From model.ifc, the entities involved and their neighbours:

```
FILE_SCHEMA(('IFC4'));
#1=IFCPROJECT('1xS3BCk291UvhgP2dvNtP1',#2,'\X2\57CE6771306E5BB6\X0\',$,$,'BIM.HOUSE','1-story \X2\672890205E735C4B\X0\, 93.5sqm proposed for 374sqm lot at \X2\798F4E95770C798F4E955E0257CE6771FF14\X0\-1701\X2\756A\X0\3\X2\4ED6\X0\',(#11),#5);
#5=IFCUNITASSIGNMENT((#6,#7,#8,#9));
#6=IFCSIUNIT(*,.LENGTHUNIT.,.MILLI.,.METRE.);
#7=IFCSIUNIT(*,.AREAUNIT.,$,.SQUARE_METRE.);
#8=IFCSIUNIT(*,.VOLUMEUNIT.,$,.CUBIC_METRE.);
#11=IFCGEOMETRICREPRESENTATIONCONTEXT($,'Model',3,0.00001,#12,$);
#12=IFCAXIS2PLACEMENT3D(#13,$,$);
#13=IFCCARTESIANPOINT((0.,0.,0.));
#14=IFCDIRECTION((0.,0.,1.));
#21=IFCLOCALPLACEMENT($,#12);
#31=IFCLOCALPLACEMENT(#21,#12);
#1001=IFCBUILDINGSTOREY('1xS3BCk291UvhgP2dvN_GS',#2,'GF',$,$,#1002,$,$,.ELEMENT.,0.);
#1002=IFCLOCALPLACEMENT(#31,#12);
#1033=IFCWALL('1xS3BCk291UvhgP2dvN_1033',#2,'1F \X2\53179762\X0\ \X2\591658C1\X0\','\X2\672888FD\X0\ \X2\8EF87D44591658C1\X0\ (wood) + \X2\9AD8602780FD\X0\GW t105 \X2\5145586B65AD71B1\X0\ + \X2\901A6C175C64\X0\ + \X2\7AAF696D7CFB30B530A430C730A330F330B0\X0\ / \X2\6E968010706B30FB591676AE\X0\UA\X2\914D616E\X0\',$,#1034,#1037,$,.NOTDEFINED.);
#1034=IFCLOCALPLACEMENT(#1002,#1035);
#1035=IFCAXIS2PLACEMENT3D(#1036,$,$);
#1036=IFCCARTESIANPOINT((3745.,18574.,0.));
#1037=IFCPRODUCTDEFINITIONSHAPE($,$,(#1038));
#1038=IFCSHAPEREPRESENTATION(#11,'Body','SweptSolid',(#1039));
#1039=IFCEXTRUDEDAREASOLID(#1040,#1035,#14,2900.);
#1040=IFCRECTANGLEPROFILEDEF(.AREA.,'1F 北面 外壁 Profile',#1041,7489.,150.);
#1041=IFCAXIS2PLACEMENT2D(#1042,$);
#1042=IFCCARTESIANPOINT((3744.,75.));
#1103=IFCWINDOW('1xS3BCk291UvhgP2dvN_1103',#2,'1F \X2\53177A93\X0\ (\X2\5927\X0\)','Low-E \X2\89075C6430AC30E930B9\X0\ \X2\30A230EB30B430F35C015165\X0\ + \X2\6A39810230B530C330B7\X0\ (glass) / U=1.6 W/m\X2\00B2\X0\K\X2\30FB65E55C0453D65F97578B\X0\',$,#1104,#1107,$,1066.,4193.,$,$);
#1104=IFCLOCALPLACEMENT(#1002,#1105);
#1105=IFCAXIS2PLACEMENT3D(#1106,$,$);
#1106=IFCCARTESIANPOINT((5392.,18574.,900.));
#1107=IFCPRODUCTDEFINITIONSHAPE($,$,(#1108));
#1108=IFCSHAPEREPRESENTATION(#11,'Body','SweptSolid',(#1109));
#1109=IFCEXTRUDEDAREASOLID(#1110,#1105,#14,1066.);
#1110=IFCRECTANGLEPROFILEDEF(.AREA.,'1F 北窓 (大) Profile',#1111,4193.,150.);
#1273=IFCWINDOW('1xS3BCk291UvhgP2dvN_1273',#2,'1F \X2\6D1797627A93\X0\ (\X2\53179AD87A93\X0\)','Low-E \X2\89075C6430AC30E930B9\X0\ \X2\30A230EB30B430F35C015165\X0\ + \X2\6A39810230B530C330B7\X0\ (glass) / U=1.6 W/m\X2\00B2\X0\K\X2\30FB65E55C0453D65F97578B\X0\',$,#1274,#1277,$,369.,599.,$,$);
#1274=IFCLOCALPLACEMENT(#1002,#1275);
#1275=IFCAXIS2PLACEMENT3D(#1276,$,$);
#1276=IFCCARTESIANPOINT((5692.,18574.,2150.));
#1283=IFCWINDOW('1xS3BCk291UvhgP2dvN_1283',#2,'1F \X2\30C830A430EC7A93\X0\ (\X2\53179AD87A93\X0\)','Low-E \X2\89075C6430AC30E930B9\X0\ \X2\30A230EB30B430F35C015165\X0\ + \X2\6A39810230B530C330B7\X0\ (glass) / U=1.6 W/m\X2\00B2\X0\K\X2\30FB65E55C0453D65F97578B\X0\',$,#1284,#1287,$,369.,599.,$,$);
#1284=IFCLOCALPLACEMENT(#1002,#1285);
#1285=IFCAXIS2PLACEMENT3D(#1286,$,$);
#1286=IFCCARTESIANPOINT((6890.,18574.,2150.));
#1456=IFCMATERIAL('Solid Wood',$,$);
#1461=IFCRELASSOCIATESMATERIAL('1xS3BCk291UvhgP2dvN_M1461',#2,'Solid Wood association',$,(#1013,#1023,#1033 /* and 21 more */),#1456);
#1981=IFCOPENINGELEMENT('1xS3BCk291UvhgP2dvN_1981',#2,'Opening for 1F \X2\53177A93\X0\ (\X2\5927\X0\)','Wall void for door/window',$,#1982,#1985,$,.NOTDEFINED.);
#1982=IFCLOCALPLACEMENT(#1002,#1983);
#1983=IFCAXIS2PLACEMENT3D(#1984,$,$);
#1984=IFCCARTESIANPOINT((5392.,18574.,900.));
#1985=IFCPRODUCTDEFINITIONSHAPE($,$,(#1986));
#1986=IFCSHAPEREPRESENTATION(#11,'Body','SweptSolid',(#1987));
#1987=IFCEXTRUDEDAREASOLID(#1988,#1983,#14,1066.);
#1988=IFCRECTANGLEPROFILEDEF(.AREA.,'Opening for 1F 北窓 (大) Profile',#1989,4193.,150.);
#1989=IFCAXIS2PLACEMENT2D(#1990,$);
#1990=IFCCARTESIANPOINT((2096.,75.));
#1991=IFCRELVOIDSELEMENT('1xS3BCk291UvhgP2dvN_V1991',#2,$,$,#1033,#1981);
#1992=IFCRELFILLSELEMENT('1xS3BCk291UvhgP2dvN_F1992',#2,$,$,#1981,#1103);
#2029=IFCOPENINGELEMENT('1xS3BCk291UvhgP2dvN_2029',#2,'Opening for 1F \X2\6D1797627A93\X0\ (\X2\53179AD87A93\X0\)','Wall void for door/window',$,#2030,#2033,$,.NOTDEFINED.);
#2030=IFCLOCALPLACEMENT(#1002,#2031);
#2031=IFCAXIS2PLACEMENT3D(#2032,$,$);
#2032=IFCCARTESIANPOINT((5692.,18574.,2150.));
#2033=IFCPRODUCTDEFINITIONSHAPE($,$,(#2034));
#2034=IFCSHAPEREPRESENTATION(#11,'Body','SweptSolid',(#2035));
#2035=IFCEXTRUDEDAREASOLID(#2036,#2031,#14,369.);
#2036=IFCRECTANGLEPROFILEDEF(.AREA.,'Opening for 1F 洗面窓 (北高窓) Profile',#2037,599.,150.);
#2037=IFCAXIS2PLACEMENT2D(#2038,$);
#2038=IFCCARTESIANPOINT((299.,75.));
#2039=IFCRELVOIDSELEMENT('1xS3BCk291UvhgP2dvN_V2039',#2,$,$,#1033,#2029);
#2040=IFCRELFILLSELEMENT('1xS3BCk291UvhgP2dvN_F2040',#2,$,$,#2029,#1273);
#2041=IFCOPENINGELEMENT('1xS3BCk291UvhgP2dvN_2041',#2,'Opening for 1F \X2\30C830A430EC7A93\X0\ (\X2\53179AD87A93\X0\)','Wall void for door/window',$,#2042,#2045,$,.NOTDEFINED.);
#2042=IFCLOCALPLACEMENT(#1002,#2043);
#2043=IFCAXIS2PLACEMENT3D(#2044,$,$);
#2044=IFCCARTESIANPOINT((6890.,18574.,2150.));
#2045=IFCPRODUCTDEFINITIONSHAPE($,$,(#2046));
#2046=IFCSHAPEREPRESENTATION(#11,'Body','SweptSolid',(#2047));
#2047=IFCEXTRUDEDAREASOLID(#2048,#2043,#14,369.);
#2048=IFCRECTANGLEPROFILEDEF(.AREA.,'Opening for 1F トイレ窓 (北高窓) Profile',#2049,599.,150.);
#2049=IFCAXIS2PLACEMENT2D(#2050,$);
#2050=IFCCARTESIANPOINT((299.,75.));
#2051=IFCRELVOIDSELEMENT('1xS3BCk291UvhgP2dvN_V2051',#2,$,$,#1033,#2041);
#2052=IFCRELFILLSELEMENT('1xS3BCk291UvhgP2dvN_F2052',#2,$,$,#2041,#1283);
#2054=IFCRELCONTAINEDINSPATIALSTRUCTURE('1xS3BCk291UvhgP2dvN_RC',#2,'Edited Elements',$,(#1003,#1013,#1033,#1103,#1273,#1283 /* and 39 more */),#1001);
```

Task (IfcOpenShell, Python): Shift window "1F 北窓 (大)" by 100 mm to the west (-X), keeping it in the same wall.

```python
import ifcopenshell
import ifcopenshell.api.geometry
import ifcopenshell.util.placement

model = ifcopenshell.open("model.ifc")

window = model.by_guid("1xS3BCk291UvhgP2dvN_1103")
opening = window.FillsVoids[0].RelatingOpeningElement
wall = opening.VoidsElements[0].RelatingBuildingElement

wall_matrix = ifcopenshell.util.placement.get_local_placement(wall.ObjectPlacement)
shift = wall_matrix[:3, 0] * -100.0
before = ifcopenshell.util.placement.get_local_placement(window.ObjectPlacement)[:3, 3].copy()

# The window is not placed relative to its opening, so move both.
for product in (opening, window):
    matrix = ifcopenshell.util.placement.get_local_placement(product.ObjectPlacement)
    matrix[:3, 3] += shift
    ifcopenshell.api.geometry.edit_object_placement(model, product=product, matrix=matrix, is_si=False)

after = ifcopenshell.util.placement.get_local_placement(window.ObjectPlacement)[:3, 3]
print("window moved by", (after - before).round(3) + 0.0)

model.write("model-out.ifc")
```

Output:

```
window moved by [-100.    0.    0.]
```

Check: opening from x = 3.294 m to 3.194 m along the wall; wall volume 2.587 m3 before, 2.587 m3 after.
